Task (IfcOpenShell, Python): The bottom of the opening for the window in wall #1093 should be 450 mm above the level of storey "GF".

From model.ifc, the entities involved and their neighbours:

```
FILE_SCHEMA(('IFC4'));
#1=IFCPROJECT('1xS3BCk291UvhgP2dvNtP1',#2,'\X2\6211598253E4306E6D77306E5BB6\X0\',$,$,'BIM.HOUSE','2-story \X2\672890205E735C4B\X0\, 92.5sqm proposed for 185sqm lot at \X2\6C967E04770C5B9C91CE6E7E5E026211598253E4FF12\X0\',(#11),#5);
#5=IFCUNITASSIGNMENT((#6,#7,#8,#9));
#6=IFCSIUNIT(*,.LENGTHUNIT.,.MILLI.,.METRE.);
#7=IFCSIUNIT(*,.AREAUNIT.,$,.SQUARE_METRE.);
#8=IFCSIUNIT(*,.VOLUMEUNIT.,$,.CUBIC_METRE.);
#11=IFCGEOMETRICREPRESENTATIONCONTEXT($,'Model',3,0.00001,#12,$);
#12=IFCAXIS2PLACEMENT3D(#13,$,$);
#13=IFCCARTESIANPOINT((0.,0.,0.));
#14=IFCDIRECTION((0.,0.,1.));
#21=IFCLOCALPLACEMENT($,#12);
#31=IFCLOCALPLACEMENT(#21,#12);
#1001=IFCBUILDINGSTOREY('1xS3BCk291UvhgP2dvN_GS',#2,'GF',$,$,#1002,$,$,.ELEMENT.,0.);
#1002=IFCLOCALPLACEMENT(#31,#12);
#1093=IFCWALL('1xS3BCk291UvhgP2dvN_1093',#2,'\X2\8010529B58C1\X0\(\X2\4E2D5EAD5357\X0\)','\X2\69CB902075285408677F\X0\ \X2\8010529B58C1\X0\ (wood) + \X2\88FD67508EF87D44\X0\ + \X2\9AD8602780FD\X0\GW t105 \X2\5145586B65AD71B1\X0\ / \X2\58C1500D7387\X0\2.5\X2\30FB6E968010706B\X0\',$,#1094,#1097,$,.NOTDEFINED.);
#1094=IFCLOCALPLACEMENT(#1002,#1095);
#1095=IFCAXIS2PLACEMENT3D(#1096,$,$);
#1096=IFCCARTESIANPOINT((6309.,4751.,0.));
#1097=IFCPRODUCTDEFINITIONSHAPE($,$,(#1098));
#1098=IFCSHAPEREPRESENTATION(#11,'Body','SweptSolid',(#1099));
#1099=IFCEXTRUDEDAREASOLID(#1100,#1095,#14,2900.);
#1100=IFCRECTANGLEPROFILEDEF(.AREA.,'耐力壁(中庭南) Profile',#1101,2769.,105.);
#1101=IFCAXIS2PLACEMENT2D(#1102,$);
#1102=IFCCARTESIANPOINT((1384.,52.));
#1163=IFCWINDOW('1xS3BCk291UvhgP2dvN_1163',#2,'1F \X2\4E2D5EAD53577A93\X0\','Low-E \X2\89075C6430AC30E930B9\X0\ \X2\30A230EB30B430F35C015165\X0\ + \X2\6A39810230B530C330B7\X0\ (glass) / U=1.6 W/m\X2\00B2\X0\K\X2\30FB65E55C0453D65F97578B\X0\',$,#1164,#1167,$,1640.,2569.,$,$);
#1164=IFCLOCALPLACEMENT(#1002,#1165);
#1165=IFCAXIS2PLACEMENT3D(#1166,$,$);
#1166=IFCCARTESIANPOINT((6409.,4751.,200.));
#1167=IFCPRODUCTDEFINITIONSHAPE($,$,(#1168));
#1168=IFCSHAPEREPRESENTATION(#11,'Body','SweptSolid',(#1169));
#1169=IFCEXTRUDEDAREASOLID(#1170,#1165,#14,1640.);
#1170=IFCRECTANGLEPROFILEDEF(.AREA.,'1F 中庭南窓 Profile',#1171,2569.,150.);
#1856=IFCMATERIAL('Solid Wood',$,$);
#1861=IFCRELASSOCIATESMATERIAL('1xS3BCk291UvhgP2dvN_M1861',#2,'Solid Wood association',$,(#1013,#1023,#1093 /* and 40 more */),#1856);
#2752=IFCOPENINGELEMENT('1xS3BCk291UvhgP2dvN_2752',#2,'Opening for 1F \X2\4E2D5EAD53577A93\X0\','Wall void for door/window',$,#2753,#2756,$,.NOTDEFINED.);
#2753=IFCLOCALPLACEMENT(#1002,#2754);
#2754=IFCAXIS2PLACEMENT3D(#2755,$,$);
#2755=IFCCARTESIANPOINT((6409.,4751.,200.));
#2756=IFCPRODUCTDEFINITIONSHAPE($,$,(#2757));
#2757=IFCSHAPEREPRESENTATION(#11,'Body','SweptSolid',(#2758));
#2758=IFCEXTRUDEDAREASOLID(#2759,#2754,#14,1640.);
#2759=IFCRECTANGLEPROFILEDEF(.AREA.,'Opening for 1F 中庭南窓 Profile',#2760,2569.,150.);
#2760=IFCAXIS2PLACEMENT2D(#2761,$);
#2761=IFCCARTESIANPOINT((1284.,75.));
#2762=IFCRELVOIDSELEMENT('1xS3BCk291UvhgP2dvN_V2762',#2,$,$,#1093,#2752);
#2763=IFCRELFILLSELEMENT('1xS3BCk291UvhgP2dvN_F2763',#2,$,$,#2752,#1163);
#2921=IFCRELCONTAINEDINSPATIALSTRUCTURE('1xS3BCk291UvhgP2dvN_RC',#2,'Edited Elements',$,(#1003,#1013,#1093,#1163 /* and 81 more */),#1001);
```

```python
import numpy as np
import ifcopenshell
import ifcopenshell.api.geometry
import ifcopenshell.geom
import ifcopenshell.util.element
import ifcopenshell.util.placement
import ifcopenshell.util.shape
import ifcopenshell.util.unit

model = ifcopenshell.open("model.ifc")
unit_scale = ifcopenshell.util.unit.calculate_unit_scale(model)

window = model.by_guid("1xS3BCk291UvhgP2dvN_1163")
opening = window.FillsVoids[0].RelatingOpeningElement
storey = ifcopenshell.util.element.get_container(window, ifc_class="IfcBuildingStorey")
level = ifcopenshell.util.placement.get_local_placement(storey.ObjectPlacement)[2, 3]

# The opening's origin need not be at the sill, so measure its lowest point.
shape = ifcopenshell.geom.create_shape(ifcopenshell.geom.settings(), opening)
bottom = ifcopenshell.util.shape.get_shape_bottom_elevation(shape, shape.geometry) / unit_scale
dz = level + 0.45 / unit_scale - bottom

shift = np.array([0.0, 0.0, dz])
# The window is not placed relative to its opening, so move both.
for product in (opening, window):
    matrix = ifcopenshell.util.placement.get_local_placement(product.ObjectPlacement)
    matrix[:3, 3] += shift
    ifcopenshell.api.geometry.edit_object_placement(model, product=product, matrix=matrix, is_si=False)

print(f"moved by {dz * unit_scale:+.3f} m")

model.write("model_rev.ifc")
```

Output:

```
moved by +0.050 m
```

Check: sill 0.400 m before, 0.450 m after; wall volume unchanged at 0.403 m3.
